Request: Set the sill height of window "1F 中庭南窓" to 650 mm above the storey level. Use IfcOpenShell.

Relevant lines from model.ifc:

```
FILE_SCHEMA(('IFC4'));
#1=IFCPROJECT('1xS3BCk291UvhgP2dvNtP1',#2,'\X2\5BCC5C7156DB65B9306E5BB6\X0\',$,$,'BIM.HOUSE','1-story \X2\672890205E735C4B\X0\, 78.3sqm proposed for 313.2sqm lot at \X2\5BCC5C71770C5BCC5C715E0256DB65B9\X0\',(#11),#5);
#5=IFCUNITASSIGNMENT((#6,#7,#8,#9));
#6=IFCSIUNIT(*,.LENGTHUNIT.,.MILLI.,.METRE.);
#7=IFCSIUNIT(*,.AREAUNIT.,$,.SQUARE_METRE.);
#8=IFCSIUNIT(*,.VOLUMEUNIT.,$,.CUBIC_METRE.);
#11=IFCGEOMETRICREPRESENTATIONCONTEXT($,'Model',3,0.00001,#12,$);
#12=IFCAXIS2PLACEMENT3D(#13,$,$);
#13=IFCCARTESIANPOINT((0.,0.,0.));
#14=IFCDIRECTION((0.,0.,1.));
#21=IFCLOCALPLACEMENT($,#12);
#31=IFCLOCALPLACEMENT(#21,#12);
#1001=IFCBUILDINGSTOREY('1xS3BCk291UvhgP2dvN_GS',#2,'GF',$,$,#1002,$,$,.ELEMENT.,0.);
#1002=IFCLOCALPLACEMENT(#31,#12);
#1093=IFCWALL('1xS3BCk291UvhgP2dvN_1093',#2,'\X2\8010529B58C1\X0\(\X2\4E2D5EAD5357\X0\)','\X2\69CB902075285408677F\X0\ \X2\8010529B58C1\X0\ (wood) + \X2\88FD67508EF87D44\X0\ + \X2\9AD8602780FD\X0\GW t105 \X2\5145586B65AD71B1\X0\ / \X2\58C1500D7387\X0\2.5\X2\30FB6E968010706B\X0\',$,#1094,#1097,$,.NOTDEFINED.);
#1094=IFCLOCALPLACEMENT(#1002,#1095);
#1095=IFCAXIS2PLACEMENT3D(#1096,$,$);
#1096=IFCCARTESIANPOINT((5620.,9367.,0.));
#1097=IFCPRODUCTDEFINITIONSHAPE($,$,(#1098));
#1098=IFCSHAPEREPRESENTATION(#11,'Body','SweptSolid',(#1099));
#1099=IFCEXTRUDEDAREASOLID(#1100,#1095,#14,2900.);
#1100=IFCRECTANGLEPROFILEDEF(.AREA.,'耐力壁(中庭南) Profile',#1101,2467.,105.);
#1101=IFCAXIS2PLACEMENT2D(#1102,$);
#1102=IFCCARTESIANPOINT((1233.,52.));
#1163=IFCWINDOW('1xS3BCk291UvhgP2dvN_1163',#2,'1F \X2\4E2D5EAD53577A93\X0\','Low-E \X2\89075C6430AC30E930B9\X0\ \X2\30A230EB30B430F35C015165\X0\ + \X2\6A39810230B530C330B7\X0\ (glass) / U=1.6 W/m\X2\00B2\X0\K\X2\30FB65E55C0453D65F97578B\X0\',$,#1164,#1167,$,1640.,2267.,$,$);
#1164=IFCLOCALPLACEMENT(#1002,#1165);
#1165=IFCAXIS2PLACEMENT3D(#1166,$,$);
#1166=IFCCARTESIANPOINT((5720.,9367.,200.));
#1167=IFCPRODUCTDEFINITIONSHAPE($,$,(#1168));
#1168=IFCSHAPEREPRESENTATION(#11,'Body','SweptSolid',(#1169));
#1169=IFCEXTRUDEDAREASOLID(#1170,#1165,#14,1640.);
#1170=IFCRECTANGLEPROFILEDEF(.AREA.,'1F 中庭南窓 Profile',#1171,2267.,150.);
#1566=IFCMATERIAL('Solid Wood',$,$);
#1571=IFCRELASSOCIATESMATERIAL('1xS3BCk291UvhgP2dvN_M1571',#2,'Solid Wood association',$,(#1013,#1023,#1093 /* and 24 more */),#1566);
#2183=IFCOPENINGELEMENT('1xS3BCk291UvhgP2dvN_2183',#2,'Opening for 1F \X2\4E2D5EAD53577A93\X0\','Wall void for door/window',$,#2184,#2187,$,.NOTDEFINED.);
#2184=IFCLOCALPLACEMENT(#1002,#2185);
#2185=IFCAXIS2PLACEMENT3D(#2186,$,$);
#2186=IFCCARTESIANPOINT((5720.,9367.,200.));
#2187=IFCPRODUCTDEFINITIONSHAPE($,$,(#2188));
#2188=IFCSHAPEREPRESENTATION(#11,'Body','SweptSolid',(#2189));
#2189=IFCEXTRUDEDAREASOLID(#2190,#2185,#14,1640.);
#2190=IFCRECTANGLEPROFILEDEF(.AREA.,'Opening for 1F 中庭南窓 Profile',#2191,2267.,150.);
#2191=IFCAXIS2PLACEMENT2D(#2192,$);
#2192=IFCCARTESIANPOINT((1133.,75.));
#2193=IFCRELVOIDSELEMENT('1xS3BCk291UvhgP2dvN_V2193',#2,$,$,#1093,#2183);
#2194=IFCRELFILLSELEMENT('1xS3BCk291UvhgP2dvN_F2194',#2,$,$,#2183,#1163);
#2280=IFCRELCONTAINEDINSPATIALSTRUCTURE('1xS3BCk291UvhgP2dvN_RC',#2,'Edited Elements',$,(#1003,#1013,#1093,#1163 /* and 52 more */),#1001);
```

```python
import numpy as np
import ifcopenshell
import ifcopenshell.api.geometry
import ifcopenshell.geom
import ifcopenshell.util.element
import ifcopenshell.util.placement
import ifcopenshell.util.shape
import ifcopenshell.util.unit

model = ifcopenshell.open("model.ifc")
unit_scale = ifcopenshell.util.unit.calculate_unit_scale(model)

window = model.by_guid("1xS3BCk291UvhgP2dvN_1163")
opening = window.FillsVoids[0].RelatingOpeningElement
storey = ifcopenshell.util.element.get_container(window, ifc_class="IfcBuildingStorey")
level = ifcopenshell.util.placement.get_local_placement(storey.ObjectPlacement)[2, 3]

# The opening's origin need not be at the sill, so measure its lowest point.
shape = ifcopenshell.geom.create_shape(ifcopenshell.geom.settings(), opening)
bottom = ifcopenshell.util.shape.get_shape_bottom_elevation(shape, shape.geometry) / unit_scale
dz = level + 0.65 / unit_scale - bottom

shift = np.array([0.0, 0.0, dz])
# The window is not placed relative to its opening, so move both.
for product in (opening, window):
    matrix = ifcopenshell.util.placement.get_local_placement(product.ObjectPlacement)
    matrix[:3, 3] += shift
    ifcopenshell.api.geometry.edit_object_placement(model, product=product, matrix=matrix, is_si=False)

print(f"moved by {dz * unit_scale:+.3f} m")

model.write("model-out.ifc")
```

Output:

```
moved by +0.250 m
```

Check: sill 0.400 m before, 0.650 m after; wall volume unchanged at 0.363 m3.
